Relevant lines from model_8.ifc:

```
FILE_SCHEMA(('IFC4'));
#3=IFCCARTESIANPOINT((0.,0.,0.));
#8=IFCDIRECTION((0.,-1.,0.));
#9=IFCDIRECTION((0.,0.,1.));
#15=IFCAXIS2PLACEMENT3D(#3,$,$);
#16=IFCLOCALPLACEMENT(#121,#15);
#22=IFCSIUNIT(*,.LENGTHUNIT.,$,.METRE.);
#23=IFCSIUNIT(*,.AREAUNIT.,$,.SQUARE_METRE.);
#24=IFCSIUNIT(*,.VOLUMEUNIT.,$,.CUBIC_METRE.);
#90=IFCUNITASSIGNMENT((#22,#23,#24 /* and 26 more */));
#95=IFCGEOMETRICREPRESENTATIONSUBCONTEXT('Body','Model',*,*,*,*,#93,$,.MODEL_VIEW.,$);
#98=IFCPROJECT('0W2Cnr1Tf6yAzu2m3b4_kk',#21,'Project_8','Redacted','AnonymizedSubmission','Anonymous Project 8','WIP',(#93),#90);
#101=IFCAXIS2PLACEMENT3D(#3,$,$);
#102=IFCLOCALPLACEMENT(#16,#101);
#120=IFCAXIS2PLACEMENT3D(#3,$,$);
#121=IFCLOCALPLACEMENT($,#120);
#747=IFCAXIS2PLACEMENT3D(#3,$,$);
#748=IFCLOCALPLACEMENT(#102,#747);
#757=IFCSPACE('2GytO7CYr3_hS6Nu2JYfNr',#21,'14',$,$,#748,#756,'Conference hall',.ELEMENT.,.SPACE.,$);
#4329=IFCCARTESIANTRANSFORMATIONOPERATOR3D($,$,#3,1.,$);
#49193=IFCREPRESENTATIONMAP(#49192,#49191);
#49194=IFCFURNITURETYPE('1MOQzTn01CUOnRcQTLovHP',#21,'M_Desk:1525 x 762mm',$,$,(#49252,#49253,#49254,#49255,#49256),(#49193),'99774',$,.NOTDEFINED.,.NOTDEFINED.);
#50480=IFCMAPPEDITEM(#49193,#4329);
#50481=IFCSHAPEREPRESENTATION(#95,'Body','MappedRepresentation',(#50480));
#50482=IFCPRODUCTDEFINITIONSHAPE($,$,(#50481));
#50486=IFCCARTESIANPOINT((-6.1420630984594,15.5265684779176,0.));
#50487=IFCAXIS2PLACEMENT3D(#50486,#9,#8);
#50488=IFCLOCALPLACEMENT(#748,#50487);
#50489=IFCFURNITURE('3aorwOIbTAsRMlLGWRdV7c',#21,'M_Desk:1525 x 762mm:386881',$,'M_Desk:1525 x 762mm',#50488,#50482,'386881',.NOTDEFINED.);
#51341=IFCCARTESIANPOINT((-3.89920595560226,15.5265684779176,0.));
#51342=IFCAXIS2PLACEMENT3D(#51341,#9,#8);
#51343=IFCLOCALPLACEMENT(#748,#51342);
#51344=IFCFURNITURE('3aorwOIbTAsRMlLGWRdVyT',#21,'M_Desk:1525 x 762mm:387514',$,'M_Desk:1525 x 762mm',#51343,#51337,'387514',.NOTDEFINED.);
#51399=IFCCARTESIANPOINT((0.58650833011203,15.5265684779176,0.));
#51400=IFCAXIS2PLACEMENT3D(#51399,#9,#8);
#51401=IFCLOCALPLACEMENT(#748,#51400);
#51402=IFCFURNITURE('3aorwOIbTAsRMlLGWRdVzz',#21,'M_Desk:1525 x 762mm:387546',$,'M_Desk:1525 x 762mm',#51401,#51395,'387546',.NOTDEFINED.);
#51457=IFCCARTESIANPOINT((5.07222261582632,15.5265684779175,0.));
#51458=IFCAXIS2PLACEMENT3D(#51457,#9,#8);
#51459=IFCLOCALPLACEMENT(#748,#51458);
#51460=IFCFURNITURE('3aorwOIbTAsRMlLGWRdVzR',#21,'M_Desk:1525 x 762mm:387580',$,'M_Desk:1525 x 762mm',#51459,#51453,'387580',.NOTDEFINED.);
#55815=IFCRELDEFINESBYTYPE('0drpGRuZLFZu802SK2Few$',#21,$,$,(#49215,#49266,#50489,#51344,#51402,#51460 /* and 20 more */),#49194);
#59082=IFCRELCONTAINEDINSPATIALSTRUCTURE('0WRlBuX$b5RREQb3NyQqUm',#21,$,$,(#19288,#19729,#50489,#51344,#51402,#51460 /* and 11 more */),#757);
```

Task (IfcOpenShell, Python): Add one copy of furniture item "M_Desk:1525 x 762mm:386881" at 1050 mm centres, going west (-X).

```python
import numpy as np
import ifcopenshell
import ifcopenshell.api.geometry
import ifcopenshell.api.root
import ifcopenshell.util.element
import ifcopenshell.util.placement
import ifcopenshell.util.unit

model = ifcopenshell.open("model_8.ifc")
unit_scale = ifcopenshell.util.unit.calculate_unit_scale(model)


def reuse_history(source, copy):
    """copy_class also copies each property set's owner history, people and application; keep the originals."""
    for rel in copy.IsDefinedBy:
        if rel.is_a("IfcRelDefinesByProperties") and (history := rel.RelatingPropertyDefinition.OwnerHistory):
            rel.RelatingPropertyDefinition.OwnerHistory = source.OwnerHistory
            ifcopenshell.util.element.remove_deep2(model, history)


source = model.by_id(50489)
base = ifcopenshell.util.placement.get_local_placement(source.ObjectPlacement)
step = np.array([-1.0, 0.0, 0.0]) * 1.05 / unit_scale

for i in range(1, 2):
    copy = ifcopenshell.api.root.copy_class(model, product=source)
    copy.Representation = ifcopenshell.util.element.copy_deep(
        model, source.Representation, exclude=["IfcGeometricRepresentationContext", "IfcRepresentationMap"]
    )
    copy.Name = "M_Desk:1525 x 762mm"
    copy.Tag = None
    reuse_history(source, copy)
    matrix = base.copy()
    matrix[:3, 3] += i * step
    print("added at", matrix[:3, 3].round(3) + 0.0)
    ifcopenshell.api.geometry.edit_object_placement(model, product=copy, matrix=matrix, is_si=False)

model.write("model_8-out.ifc")
```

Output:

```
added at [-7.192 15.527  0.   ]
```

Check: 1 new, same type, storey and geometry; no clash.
